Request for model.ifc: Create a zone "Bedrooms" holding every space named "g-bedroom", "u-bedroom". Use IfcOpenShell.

First a look at what the model holds.

```python
import ifcopenshell

model = ifcopenshell.open("model.ifc")
print(model.schema)
seen = {}
for space in model.by_type("IfcSpace"):
    seen[space.LongName] = seen.get(space.LongName, 0) + 1
for name, count in sorted(seen.items(), key=str):
    print(count, "x", name)
print("zones:", [z.Name for z in model.by_type("IfcZone")][:20])
```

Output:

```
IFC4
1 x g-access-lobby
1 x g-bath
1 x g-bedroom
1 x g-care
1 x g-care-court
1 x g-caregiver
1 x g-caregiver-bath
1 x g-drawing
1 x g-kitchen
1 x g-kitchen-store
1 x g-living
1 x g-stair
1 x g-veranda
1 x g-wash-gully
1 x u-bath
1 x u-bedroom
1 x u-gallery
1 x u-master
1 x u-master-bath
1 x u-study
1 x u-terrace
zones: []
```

```python
import ifcopenshell
import ifcopenshell.api.group
import ifcopenshell.api.root

model = ifcopenshell.open("model.ifc")

names = {"g-bedroom", "u-bedroom"}
spaces = [s for s in model.by_type("IfcSpace") if s.LongName in names]

zone = ifcopenshell.api.root.create_entity(model, ifc_class="IfcZone", name="Bedrooms")
ifcopenshell.api.group.assign_group(model, products=spaces, group=zone)
print(len(spaces), "spaces in", zone.Name)

model.write("model_rev.ifc")
```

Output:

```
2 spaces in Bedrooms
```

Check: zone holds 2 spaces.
